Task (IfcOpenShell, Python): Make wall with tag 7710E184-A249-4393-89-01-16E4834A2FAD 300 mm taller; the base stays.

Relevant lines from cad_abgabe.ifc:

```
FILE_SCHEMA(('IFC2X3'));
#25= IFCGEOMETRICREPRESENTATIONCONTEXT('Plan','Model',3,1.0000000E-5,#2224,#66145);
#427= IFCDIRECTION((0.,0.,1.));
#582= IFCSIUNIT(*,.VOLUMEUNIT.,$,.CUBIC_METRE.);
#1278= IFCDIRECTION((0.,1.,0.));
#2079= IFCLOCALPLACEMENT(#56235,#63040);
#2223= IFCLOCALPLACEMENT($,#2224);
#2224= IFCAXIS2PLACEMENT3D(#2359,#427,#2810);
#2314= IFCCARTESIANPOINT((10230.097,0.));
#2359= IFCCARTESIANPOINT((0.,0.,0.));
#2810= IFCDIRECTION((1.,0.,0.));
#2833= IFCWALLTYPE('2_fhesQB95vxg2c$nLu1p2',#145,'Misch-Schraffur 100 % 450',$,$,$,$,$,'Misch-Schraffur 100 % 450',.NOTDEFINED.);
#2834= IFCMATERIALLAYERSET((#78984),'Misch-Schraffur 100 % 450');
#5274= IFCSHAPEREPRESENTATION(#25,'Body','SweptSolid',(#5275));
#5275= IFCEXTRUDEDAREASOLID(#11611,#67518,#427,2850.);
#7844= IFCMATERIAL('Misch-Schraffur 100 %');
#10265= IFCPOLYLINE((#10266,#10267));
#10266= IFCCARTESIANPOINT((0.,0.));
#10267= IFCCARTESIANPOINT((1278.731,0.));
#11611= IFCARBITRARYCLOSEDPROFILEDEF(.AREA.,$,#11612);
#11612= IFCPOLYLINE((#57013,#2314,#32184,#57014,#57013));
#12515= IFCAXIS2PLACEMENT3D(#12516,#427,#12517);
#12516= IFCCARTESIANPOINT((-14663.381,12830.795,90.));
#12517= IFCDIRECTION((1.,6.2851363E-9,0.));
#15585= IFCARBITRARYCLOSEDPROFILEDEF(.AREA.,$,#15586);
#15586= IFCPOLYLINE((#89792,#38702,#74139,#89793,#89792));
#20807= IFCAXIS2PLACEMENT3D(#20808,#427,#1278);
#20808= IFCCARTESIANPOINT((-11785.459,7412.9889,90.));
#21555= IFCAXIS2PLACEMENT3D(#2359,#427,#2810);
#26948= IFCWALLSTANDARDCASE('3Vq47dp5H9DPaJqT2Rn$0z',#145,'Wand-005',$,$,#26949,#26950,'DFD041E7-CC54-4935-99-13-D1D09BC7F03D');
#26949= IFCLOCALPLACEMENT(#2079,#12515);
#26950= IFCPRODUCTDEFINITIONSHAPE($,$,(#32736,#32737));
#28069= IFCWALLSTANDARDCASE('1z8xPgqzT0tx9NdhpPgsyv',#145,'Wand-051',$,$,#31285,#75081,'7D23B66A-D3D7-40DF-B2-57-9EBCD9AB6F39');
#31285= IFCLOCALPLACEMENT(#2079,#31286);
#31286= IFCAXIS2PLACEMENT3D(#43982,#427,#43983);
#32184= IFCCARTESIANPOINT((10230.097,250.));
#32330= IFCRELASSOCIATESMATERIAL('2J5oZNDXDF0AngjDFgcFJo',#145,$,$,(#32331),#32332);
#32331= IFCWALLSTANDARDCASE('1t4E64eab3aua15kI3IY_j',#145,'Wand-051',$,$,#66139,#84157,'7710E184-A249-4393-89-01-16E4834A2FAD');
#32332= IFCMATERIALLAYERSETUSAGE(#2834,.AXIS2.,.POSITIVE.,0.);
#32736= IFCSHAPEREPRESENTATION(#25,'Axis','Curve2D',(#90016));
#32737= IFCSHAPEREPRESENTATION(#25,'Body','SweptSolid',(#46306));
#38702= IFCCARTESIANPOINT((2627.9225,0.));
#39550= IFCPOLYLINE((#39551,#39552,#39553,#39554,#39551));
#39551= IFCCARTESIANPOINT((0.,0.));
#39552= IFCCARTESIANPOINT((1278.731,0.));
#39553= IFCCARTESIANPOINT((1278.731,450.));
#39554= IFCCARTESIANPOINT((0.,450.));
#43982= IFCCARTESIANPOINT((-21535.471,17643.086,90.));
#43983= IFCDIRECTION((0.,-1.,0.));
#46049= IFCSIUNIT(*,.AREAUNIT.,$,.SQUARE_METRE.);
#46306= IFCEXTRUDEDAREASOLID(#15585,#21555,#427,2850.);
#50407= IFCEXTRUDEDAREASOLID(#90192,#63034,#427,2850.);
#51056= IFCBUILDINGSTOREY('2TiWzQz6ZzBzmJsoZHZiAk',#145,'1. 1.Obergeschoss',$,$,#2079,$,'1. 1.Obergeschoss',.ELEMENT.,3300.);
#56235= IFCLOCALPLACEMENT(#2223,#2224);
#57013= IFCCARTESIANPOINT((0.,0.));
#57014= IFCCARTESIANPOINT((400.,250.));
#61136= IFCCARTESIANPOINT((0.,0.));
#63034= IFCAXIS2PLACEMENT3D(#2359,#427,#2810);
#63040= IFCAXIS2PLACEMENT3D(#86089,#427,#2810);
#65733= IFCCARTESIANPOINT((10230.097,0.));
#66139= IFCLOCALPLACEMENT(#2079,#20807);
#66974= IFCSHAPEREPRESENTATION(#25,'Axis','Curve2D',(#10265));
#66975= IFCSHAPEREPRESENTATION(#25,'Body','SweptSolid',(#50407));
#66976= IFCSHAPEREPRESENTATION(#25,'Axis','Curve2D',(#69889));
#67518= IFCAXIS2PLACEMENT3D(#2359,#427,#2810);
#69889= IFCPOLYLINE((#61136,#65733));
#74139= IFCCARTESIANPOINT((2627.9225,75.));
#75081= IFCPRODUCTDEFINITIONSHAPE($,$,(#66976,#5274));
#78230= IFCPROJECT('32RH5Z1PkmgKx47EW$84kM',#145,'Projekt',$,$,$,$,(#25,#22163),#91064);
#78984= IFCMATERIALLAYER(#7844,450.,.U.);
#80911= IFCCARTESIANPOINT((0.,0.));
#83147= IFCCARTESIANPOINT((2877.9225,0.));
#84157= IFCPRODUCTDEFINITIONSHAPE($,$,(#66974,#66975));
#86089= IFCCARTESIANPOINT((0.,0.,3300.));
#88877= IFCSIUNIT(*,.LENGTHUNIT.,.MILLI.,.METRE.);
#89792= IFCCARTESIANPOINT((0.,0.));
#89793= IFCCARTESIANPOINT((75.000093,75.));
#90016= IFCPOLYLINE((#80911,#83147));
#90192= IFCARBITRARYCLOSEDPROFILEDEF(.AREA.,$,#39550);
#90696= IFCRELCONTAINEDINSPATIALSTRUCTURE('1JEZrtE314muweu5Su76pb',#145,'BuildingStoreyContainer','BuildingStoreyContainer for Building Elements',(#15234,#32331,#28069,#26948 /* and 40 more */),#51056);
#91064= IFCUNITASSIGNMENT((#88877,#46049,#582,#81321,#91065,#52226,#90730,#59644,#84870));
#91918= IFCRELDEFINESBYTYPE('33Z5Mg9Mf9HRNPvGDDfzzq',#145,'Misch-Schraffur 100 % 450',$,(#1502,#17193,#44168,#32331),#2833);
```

```python
import ifcopenshell
import ifcopenshell.geom
import ifcopenshell.util.shape
import ifcopenshell.util.unit

model = ifcopenshell.open("cad_abgabe.ifc")
unit_scale = ifcopenshell.util.unit.calculate_unit_scale(model)
settings = ifcopenshell.geom.settings()


def volume(element):
    """Net volume in cubic metres, openings subtracted."""
    shape = ifcopenshell.geom.create_shape(settings, element)
    return ifcopenshell.util.shape.get_volume(shape.geometry)


wall = model.by_id(32331)
before = volume(wall)

body = next(r for r in wall.Representation.Representations if r.RepresentationIdentifier == "Body")
solid = body.Items[0]
old_height = solid.Depth
solid.Depth += 0.3 / unit_scale
after = volume(wall)

print(f"height {old_height:g} -> {solid.Depth:g}, volume {before:.3f} -> {after:.3f} m3")

model.write("cad_abgabe_rev.ifc")
```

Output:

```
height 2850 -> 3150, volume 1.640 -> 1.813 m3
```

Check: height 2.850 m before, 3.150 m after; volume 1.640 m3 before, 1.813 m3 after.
